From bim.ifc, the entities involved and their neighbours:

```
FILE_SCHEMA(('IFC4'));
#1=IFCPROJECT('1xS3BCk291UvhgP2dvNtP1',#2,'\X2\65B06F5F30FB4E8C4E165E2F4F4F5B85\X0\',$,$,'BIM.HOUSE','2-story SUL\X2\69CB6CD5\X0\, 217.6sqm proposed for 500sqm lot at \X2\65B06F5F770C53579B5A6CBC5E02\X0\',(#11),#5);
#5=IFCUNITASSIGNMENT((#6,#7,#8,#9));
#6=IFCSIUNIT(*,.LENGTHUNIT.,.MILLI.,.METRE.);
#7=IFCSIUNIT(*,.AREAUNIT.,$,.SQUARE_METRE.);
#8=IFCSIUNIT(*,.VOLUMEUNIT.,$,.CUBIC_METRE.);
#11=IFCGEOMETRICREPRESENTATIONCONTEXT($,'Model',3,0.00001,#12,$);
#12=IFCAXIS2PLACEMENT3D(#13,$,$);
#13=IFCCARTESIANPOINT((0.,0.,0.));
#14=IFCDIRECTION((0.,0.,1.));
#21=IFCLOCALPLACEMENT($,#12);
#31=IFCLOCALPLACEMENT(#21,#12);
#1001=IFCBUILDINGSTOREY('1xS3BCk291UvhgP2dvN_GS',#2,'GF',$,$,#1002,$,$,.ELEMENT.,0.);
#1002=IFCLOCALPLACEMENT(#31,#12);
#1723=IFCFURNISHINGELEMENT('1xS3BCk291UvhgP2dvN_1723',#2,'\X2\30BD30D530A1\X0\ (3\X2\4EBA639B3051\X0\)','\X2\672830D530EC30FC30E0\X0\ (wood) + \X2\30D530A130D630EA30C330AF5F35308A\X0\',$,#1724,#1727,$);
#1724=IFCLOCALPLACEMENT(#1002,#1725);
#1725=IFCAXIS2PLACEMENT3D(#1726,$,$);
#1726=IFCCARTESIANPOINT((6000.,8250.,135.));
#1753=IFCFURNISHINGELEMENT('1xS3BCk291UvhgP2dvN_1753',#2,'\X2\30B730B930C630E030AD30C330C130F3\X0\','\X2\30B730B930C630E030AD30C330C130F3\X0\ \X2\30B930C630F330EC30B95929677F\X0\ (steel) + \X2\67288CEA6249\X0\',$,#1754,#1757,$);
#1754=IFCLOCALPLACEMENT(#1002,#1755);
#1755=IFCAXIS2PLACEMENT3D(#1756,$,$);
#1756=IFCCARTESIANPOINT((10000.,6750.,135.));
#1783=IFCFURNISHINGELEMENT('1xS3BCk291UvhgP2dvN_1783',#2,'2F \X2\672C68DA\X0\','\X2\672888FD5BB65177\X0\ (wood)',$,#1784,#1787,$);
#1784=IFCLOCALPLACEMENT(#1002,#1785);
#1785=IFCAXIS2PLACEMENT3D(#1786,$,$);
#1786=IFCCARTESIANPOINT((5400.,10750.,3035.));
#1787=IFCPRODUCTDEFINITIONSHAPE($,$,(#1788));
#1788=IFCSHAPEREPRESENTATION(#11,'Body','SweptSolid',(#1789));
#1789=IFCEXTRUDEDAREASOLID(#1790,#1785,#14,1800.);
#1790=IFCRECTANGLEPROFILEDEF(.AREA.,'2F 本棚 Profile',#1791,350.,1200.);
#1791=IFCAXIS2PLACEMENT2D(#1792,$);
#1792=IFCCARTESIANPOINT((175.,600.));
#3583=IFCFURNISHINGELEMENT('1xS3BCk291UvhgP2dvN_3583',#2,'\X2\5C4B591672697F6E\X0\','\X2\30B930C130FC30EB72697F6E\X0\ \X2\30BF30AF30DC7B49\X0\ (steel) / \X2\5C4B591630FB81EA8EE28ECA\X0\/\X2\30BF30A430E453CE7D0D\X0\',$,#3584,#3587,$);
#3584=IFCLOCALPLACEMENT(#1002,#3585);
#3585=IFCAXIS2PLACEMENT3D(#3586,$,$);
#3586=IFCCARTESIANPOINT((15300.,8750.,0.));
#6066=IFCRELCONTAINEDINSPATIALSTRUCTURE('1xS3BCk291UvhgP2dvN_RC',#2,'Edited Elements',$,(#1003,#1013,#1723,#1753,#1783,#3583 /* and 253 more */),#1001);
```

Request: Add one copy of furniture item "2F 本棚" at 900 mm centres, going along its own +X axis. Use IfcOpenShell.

```python
import ifcopenshell
import ifcopenshell.api.geometry
import ifcopenshell.api.root
import ifcopenshell.util.element
import ifcopenshell.util.placement
import ifcopenshell.util.unit

model = ifcopenshell.open("bim.ifc")
unit_scale = ifcopenshell.util.unit.calculate_unit_scale(model)


def reuse_history(source, copy):
    """copy_class also copies each property set's owner history, people and application; keep the originals."""
    for rel in copy.IsDefinedBy:
        if rel.is_a("IfcRelDefinesByProperties") and (history := rel.RelatingPropertyDefinition.OwnerHistory):
            rel.RelatingPropertyDefinition.OwnerHistory = source.OwnerHistory
            ifcopenshell.util.element.remove_deep2(model, history)


source = model.by_guid("1xS3BCk291UvhgP2dvN_1783")
base = ifcopenshell.util.placement.get_local_placement(source.ObjectPlacement)
step = base[:3, 0] * 0.9 / unit_scale

for i in range(1, 2):
    copy = ifcopenshell.api.root.copy_class(model, product=source)
    copy.Representation = ifcopenshell.util.element.copy_deep(
        model, source.Representation, exclude=["IfcGeometricRepresentationContext", "IfcRepresentationMap"]
    )
    reuse_history(source, copy)
    matrix = base.copy()
    matrix[:3, 3] += i * step
    print("added at", matrix[:3, 3].round(3) + 0.0)
    ifcopenshell.api.geometry.edit_object_placement(model, product=copy, matrix=matrix, is_si=False)

model.write("bim_rev.ifc")
```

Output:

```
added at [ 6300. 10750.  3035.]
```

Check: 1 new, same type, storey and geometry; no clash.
